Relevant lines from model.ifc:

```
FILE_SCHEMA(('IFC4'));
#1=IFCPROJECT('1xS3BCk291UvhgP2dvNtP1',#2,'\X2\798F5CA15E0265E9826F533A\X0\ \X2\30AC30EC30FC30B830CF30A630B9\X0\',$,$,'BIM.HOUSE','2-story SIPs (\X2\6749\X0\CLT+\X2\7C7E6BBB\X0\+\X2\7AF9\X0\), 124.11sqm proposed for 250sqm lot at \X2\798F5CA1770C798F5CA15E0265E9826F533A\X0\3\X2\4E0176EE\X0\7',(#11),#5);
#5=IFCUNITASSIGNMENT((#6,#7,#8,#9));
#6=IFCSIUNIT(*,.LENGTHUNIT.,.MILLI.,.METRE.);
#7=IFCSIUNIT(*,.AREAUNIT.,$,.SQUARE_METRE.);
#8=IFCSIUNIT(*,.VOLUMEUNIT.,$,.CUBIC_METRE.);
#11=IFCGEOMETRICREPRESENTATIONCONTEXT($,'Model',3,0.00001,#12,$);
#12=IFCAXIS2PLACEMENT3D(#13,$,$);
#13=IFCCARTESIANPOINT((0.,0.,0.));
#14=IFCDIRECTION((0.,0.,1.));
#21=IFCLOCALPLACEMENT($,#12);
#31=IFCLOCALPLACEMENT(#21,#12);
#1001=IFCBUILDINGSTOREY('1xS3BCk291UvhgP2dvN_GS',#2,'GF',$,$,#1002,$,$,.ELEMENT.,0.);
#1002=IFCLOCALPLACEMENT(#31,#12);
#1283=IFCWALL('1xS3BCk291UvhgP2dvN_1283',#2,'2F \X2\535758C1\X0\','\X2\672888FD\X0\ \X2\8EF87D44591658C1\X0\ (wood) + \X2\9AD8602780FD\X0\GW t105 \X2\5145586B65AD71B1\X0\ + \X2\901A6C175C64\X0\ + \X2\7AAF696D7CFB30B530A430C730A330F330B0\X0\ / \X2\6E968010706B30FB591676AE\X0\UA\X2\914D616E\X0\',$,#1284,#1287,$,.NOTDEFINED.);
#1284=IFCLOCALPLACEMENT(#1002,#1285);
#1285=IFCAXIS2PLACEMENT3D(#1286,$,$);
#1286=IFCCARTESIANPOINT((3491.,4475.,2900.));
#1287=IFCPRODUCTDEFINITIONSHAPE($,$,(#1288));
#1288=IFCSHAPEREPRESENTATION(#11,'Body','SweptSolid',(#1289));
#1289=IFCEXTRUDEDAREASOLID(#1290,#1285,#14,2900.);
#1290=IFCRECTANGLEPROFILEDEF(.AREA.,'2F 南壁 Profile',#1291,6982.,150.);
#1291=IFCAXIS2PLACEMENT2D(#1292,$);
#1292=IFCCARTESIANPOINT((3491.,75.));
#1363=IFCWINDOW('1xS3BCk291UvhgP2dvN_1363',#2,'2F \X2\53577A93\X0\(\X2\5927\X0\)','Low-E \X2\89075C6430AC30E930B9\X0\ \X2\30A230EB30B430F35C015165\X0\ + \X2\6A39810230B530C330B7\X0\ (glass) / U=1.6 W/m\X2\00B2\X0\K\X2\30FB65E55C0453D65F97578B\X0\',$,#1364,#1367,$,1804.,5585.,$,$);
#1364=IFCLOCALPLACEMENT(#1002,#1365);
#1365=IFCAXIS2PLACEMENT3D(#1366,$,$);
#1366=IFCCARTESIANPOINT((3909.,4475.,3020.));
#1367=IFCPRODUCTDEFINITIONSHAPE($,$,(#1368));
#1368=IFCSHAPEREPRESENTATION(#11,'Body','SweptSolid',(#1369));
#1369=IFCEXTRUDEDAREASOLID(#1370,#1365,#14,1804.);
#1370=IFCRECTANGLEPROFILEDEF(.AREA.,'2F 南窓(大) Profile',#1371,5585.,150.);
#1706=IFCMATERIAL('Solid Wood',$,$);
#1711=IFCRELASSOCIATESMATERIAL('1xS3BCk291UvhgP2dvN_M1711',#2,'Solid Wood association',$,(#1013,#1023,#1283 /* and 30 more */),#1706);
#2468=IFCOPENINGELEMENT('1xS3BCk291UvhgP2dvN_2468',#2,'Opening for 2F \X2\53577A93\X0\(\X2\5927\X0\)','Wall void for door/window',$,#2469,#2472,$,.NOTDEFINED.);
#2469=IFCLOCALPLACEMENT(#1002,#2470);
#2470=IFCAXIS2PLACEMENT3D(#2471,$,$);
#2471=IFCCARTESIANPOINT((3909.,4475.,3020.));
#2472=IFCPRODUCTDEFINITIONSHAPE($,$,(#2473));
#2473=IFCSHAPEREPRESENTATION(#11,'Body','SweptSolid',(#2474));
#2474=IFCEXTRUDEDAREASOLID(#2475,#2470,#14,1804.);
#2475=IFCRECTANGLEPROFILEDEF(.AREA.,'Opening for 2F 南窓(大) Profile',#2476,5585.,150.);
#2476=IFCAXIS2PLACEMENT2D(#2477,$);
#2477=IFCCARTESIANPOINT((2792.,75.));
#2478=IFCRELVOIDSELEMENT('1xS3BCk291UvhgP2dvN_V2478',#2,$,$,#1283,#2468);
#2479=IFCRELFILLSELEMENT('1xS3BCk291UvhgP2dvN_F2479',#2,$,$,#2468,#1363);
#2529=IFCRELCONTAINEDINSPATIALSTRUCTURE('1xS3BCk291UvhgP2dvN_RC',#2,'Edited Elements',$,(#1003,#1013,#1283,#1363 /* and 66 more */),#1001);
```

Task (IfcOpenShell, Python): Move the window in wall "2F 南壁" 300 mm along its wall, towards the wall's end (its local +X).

```python
import ifcopenshell
import ifcopenshell.api.geometry
import ifcopenshell.util.placement
import ifcopenshell.util.unit

model = ifcopenshell.open("model.ifc")
unit_scale = ifcopenshell.util.unit.calculate_unit_scale(model)

window = model.by_id(1363)
opening = window.FillsVoids[0].RelatingOpeningElement
wall = opening.VoidsElements[0].RelatingBuildingElement

wall_matrix = ifcopenshell.util.placement.get_local_placement(wall.ObjectPlacement)
shift = wall_matrix[:3, 0] * 0.3 / unit_scale
before = ifcopenshell.util.placement.get_local_placement(window.ObjectPlacement)[:3, 3].copy()

# The window is not placed relative to its opening, so move both.
for product in (opening, window):
    matrix = ifcopenshell.util.placement.get_local_placement(product.ObjectPlacement)
    matrix[:3, 3] += shift
    ifcopenshell.api.geometry.edit_object_placement(model, product=product, matrix=matrix, is_si=False)

after = ifcopenshell.util.placement.get_local_placement(window.ObjectPlacement)[:3, 3]
print("window moved by", (after - before).round(3) + 0.0)

model.write("model-out.ifc")
```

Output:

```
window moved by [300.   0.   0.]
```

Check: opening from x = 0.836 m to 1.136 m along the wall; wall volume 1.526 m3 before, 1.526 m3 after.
